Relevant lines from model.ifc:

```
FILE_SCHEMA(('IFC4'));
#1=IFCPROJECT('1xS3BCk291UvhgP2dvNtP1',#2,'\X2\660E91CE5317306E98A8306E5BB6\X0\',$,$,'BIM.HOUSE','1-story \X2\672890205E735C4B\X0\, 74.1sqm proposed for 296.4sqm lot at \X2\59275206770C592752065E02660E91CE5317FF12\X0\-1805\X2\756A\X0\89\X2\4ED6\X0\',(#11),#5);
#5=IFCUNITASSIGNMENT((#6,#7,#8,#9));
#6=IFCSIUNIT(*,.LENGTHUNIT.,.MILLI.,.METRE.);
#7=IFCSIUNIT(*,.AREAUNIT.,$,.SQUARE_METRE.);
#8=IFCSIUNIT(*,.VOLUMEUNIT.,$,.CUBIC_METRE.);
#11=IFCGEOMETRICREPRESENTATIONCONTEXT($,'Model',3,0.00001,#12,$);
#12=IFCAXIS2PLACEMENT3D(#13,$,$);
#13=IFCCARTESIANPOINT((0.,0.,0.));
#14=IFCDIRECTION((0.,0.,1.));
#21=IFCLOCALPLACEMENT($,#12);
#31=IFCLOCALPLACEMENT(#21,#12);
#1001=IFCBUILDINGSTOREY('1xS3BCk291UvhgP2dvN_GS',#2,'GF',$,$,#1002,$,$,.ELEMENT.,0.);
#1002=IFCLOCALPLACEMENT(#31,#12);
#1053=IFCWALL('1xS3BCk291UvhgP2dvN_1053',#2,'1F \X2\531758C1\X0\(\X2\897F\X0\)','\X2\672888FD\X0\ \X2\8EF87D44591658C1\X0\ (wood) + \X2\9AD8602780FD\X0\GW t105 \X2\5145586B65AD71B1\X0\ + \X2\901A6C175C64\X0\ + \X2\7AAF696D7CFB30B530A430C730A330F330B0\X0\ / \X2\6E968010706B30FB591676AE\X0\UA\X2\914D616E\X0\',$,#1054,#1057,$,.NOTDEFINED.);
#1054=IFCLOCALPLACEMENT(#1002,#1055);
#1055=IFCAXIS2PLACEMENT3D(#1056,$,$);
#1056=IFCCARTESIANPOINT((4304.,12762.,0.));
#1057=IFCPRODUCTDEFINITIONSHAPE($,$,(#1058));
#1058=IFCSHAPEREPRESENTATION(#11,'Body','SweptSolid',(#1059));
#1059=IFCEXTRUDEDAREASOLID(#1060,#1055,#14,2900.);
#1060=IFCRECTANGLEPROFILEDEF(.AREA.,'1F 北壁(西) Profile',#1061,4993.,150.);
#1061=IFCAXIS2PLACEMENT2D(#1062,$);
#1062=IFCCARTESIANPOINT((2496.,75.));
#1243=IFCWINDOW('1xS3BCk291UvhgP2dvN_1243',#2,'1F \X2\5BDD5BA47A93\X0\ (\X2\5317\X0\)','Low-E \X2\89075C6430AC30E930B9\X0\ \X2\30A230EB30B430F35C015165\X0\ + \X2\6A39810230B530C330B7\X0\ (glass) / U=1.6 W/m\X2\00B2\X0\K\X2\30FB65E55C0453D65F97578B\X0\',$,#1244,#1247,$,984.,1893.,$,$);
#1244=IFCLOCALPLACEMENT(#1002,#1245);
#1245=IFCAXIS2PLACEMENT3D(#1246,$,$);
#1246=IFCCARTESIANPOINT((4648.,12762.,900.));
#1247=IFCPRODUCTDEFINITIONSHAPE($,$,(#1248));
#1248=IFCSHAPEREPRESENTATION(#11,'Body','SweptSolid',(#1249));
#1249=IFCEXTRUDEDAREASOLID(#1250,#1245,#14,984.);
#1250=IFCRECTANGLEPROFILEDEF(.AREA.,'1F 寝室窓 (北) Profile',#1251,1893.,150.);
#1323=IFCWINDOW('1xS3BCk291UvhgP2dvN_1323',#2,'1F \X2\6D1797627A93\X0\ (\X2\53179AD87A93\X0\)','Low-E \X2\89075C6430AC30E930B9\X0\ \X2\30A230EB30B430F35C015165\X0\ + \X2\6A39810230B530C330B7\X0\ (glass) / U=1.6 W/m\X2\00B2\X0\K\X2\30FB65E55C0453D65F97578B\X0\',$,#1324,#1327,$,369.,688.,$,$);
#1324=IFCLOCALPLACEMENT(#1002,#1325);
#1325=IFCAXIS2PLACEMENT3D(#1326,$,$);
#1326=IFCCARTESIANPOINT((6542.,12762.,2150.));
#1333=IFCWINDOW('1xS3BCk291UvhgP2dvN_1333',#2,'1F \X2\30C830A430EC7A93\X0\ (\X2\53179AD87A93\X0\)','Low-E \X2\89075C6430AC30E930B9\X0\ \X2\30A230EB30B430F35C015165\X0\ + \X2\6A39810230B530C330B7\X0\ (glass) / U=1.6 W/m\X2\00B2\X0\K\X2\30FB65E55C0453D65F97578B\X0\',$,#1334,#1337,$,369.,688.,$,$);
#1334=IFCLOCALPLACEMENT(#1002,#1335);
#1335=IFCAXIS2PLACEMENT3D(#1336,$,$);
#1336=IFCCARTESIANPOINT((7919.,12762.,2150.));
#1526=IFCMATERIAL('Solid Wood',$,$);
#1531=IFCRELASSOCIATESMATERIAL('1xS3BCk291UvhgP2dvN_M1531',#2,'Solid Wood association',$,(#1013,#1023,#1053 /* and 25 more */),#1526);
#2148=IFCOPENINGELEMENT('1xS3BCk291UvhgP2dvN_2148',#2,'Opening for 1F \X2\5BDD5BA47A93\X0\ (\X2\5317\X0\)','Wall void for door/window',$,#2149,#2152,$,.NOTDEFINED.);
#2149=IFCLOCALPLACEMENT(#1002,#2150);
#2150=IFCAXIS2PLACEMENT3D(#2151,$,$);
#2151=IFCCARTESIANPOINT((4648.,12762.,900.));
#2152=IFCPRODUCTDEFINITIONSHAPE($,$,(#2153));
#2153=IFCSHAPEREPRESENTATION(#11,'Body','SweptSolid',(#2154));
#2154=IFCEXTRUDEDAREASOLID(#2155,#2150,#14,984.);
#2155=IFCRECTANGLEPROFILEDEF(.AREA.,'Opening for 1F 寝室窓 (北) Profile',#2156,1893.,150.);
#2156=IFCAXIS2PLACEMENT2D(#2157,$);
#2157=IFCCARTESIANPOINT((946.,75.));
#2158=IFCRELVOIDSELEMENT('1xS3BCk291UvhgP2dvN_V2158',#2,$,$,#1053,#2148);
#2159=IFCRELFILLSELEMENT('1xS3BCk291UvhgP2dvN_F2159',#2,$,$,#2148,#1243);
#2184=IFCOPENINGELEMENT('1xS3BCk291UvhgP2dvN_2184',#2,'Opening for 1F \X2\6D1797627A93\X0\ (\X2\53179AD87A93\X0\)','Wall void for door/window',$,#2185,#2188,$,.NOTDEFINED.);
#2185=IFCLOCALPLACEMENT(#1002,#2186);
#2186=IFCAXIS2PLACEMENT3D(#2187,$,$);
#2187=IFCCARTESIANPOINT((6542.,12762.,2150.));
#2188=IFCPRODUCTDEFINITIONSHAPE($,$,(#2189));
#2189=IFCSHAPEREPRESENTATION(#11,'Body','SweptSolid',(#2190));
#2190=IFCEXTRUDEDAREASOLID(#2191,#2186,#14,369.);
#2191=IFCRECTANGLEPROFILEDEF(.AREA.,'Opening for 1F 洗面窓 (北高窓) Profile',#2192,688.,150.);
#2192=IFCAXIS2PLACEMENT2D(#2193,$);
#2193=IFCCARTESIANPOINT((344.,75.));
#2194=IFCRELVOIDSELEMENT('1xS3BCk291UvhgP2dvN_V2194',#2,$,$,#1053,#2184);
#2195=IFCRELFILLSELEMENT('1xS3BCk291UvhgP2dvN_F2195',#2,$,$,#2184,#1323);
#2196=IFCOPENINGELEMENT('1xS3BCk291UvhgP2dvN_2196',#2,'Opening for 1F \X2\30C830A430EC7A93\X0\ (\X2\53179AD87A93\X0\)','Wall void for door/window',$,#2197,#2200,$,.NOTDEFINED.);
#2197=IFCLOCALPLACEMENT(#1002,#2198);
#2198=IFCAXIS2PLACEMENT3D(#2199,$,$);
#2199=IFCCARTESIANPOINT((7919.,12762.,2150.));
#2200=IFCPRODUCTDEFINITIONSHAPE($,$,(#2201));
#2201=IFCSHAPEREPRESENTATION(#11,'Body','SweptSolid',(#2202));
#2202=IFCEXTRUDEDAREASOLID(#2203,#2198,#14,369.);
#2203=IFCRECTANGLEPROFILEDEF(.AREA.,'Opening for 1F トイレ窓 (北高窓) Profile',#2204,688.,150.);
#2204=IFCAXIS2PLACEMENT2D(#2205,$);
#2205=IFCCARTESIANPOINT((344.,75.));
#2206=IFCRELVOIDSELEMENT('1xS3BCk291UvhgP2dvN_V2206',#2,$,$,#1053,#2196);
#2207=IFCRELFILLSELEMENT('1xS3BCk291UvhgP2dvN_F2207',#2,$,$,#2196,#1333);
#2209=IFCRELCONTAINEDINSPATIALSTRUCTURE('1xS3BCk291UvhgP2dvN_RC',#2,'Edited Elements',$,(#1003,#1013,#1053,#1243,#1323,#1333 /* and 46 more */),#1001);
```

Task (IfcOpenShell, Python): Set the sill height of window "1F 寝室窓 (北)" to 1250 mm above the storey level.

```python
import numpy as np
import ifcopenshell
import ifcopenshell.api.geometry
import ifcopenshell.geom
import ifcopenshell.util.element
import ifcopenshell.util.placement
import ifcopenshell.util.shape
import ifcopenshell.util.unit

model = ifcopenshell.open("model.ifc")
unit_scale = ifcopenshell.util.unit.calculate_unit_scale(model)

window = model.by_guid("1xS3BCk291UvhgP2dvN_1243")
opening = window.FillsVoids[0].RelatingOpeningElement
storey = ifcopenshell.util.element.get_container(window, ifc_class="IfcBuildingStorey")
level = ifcopenshell.util.placement.get_local_placement(storey.ObjectPlacement)[2, 3]

# The opening's origin need not be at the sill, so measure its lowest point.
shape = ifcopenshell.geom.create_shape(ifcopenshell.geom.settings(), opening)
bottom = ifcopenshell.util.shape.get_shape_bottom_elevation(shape, shape.geometry) / unit_scale
dz = level + 1.25 / unit_scale - bottom

shift = np.array([0.0, 0.0, dz])
# The window is not placed relative to its opening, so move both.
for product in (opening, window):
    matrix = ifcopenshell.util.placement.get_local_placement(product.ObjectPlacement)
    matrix[:3, 3] += shift
    ifcopenshell.api.geometry.edit_object_placement(model, product=product, matrix=matrix, is_si=False)

print(f"moved by {dz * unit_scale:+.3f} m")

model.write("model-out.ifc")
```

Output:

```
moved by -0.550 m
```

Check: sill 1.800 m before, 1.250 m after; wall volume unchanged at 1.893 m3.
